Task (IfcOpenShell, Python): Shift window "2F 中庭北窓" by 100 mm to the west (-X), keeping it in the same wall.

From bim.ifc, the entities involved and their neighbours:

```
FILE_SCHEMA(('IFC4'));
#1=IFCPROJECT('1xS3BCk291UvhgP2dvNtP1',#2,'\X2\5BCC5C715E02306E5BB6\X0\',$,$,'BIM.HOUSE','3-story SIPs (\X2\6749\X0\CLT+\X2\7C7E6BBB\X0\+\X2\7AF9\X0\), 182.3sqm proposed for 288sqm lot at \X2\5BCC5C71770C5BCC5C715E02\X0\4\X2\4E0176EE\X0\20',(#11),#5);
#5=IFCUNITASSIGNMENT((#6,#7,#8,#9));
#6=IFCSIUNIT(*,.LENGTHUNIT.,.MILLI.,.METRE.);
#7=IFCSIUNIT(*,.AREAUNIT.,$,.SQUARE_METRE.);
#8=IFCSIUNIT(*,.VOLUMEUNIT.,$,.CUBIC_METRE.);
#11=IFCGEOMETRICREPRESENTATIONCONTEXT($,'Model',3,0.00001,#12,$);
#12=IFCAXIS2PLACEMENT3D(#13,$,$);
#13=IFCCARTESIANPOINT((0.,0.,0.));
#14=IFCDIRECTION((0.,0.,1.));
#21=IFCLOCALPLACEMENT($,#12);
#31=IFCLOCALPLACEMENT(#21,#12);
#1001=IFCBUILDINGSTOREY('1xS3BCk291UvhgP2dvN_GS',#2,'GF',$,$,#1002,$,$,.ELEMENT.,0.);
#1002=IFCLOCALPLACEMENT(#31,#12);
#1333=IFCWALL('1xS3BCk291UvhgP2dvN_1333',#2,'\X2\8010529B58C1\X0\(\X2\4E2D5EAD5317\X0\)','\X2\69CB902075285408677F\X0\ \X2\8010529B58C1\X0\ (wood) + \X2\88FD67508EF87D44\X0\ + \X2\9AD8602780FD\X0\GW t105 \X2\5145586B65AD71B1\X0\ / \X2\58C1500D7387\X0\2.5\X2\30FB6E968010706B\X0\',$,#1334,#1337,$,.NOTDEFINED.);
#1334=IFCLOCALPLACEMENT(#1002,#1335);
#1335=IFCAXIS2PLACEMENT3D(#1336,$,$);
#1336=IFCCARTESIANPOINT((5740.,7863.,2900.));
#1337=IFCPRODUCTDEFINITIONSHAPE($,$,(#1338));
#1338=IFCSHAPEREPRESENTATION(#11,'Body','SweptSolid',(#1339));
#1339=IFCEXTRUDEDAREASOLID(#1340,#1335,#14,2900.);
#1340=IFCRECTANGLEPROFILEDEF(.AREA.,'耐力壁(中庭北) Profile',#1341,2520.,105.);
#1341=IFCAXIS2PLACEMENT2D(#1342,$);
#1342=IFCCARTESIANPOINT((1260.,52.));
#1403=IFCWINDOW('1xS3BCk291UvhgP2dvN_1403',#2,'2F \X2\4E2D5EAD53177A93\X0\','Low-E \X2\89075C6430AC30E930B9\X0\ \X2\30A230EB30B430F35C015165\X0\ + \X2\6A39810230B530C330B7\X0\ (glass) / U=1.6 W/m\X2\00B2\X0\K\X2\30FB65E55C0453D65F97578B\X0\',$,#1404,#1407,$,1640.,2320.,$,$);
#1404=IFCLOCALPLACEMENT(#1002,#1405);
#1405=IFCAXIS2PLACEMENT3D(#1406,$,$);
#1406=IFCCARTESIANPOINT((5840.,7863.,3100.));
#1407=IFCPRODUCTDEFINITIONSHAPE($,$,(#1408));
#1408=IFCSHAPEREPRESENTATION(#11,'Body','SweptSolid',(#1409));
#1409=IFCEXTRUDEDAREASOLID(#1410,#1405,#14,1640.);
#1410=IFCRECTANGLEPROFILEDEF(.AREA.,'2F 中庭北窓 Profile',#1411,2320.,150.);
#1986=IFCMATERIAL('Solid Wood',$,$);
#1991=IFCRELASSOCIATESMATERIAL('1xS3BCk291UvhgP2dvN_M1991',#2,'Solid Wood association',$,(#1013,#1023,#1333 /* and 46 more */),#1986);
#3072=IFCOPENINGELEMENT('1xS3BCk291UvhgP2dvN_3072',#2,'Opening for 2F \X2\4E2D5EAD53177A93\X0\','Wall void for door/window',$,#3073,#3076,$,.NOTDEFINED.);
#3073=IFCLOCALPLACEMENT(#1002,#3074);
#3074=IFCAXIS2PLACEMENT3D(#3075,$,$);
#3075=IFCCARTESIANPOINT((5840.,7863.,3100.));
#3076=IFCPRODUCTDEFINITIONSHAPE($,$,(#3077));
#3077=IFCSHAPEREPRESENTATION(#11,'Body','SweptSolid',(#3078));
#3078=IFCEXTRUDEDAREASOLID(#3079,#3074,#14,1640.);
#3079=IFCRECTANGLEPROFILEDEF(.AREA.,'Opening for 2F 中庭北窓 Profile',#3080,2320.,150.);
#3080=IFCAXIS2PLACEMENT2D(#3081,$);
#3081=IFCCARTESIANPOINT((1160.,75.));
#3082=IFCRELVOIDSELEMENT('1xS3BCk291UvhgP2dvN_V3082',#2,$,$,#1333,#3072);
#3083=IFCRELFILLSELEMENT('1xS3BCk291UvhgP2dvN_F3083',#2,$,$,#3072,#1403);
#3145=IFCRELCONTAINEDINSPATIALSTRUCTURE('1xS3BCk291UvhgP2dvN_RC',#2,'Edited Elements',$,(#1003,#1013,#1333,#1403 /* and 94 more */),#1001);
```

```python
import ifcopenshell
import ifcopenshell.api.geometry
import ifcopenshell.util.placement

model = ifcopenshell.open("bim.ifc")

window = model.by_guid("1xS3BCk291UvhgP2dvN_1403")
opening = window.FillsVoids[0].RelatingOpeningElement
wall = opening.VoidsElements[0].RelatingBuildingElement

wall_matrix = ifcopenshell.util.placement.get_local_placement(wall.ObjectPlacement)
shift = wall_matrix[:3, 0] * -100.0
before = ifcopenshell.util.placement.get_local_placement(window.ObjectPlacement)[:3, 3].copy()

# The window is not placed relative to its opening, so move both.
for product in (opening, window):
    matrix = ifcopenshell.util.placement.get_local_placement(product.ObjectPlacement)
    matrix[:3, 3] += shift
    ifcopenshell.api.geometry.edit_object_placement(model, product=product, matrix=matrix, is_si=False)

after = ifcopenshell.util.placement.get_local_placement(window.ObjectPlacement)[:3, 3]
print("window moved by", (after - before).round(3) + 0.0)

model.write("bim-out.ifc")
```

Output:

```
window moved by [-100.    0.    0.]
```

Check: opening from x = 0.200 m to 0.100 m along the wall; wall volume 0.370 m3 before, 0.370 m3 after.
